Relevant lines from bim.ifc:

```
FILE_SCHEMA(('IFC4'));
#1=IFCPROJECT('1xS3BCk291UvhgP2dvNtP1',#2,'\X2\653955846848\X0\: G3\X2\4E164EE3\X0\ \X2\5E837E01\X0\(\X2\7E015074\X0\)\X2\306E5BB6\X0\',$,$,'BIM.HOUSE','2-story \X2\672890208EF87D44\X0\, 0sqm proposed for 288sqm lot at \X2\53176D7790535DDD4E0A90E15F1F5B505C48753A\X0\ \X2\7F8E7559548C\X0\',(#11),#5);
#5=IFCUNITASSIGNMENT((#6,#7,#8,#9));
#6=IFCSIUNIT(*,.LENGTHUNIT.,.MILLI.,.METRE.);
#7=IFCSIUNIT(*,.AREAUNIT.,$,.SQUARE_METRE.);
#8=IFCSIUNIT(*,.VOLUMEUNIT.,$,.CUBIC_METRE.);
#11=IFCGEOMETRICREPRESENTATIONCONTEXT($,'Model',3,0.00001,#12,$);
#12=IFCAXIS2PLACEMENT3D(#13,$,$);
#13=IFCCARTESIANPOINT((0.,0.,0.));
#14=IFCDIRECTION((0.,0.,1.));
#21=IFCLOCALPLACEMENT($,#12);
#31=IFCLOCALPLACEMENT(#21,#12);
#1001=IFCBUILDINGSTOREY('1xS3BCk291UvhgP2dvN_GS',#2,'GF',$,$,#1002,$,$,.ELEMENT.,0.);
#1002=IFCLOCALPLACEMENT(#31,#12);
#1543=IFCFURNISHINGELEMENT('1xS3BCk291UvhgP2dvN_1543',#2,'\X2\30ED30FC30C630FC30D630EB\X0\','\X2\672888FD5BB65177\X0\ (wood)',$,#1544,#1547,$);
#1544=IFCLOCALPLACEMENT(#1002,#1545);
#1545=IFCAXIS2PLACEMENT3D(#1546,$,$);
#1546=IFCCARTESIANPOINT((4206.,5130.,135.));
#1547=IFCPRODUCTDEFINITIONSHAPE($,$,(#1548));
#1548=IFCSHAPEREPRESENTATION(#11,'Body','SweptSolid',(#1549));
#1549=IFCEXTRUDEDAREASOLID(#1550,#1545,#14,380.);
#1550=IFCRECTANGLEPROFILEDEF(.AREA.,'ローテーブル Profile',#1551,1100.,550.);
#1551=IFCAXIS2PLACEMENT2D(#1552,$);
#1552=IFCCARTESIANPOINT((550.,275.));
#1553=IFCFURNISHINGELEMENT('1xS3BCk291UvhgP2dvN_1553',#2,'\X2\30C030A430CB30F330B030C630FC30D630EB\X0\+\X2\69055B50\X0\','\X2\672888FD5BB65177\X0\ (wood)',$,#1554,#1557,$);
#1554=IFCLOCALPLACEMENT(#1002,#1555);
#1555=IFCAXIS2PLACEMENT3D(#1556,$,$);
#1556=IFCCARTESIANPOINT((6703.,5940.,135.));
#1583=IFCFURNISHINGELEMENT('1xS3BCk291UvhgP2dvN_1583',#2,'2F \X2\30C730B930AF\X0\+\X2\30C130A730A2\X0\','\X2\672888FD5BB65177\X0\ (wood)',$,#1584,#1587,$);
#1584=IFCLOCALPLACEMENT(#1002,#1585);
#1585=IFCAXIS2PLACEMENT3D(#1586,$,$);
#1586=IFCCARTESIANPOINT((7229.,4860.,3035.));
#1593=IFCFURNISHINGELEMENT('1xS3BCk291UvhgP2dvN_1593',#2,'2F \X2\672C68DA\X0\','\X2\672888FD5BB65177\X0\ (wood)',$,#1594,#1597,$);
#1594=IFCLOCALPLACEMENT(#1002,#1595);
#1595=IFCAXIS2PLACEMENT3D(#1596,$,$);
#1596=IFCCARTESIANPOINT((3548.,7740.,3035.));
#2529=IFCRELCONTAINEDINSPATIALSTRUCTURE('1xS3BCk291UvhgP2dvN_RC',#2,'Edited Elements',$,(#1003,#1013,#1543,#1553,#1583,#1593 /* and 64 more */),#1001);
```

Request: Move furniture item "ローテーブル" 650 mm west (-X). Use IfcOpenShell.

```python
import ifcopenshell
import ifcopenshell.api.geometry
import ifcopenshell.util.placement

model = ifcopenshell.open("bim.ifc")

item = model.by_guid("1xS3BCk291UvhgP2dvN_1543")
matrix = ifcopenshell.util.placement.get_local_placement(item.ObjectPlacement)
matrix[0, 3] -= 650.0
ifcopenshell.api.geometry.edit_object_placement(model, product=item, matrix=matrix, is_si=False)

print(ifcopenshell.util.placement.get_local_placement(item.ObjectPlacement).round(3) + 0.0)

model.write("bim_v2.ifc")
```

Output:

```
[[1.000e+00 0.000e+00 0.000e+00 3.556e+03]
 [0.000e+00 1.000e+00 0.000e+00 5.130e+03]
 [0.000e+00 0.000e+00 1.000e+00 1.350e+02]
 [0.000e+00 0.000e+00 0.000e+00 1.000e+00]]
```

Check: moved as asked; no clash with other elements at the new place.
